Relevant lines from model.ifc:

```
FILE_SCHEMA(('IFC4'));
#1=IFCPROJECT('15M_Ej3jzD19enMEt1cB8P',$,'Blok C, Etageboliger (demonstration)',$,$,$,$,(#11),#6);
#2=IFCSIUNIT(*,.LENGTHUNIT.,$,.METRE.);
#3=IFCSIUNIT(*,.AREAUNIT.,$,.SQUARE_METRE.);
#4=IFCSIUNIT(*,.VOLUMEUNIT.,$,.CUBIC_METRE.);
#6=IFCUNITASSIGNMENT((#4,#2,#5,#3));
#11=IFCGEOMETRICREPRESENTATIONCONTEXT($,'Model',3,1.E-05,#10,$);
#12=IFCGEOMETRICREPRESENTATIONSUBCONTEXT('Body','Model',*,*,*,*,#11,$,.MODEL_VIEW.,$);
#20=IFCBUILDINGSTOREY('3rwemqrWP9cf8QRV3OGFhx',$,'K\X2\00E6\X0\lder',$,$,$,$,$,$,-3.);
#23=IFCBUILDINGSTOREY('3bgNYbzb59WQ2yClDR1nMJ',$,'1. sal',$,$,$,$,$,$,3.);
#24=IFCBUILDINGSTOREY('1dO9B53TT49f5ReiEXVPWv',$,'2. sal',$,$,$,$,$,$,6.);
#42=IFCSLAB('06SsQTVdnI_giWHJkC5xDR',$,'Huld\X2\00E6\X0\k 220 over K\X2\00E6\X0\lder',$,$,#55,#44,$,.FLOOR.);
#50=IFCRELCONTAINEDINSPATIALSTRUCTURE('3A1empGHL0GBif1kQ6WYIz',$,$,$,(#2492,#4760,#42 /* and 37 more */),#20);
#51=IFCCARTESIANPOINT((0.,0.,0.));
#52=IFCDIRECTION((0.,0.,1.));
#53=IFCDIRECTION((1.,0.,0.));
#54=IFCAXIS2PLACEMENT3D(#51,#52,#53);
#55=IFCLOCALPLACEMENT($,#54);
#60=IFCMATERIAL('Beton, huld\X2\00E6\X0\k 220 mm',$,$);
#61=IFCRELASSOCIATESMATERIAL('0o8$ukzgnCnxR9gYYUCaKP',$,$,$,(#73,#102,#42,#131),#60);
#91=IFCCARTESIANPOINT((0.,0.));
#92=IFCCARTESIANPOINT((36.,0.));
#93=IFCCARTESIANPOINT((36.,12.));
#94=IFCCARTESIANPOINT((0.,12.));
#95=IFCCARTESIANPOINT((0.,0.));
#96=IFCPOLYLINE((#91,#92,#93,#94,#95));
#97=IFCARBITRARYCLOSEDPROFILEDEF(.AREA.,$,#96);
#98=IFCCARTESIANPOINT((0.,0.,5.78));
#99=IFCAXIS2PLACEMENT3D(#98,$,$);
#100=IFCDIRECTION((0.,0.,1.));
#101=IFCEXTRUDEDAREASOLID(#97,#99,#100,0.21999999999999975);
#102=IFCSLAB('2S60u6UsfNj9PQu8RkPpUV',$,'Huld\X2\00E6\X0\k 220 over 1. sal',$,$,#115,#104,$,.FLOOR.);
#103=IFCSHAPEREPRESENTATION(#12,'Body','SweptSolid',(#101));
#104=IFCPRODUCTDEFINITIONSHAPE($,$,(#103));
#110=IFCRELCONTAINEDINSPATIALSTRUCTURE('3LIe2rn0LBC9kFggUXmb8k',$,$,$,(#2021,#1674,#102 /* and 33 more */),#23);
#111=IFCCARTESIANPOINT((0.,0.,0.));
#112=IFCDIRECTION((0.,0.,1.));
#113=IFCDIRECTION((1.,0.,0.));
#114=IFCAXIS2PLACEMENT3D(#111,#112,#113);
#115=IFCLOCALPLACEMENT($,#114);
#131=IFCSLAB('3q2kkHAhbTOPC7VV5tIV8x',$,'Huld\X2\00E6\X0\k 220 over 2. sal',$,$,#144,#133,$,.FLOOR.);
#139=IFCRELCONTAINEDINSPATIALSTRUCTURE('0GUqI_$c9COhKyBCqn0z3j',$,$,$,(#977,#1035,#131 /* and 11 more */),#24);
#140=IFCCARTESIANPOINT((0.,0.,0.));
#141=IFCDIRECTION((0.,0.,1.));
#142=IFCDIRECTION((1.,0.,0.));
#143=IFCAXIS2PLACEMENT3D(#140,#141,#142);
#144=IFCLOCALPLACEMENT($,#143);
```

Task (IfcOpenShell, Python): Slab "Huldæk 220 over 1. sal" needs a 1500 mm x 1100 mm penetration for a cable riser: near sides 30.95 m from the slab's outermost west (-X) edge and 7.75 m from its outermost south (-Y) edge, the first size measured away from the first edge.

```python
import numpy as np
import ifcopenshell
import ifcopenshell.api.feature
import ifcopenshell.api.geometry
import ifcopenshell.api.root
import ifcopenshell.geom
import ifcopenshell.util.placement
import ifcopenshell.util.representation
import ifcopenshell.util.shape
import ifcopenshell.util.unit

model = ifcopenshell.open("model.ifc")
unit_scale = ifcopenshell.util.unit.calculate_unit_scale(model)
settings = ifcopenshell.geom.settings()


def volume(element):
    """Net volume in cubic metres, openings subtracted."""
    shape = ifcopenshell.geom.create_shape(settings, element)
    return ifcopenshell.util.shape.get_volume(shape.geometry)


slab = model.by_id(102)
before = volume(slab)

# Extent in the slab's own axes, in metres. The edges named are its -X and -Y sides.
slab_shape = ifcopenshell.geom.create_shape(settings, slab)
vertices = ifcopenshell.util.shape.get_vertices(slab_shape.geometry)
x_min, y_min, bottom = vertices.min(axis=0)
top = vertices[:, 2].max()

opening = ifcopenshell.api.root.create_entity(model, ifc_class="IfcOpeningElement", name="Cable riser opening", predefined_type="OPENING")
context = ifcopenshell.util.representation.get_context(model, "Model", "Body", "MODEL_VIEW")
width, depth = 1.5, 1.1
outline = [(0.0, 0.0), (width, 0.0), (width, depth), (0.0, depth), (0.0, 0.0)]
# Overshoot both faces by 50 mm so the cut is clean.
shape = ifcopenshell.api.geometry.add_slab_representation(
    model, context=context, depth=top - bottom + 0.1, polyline=outline
)
ifcopenshell.api.geometry.assign_representation(model, product=opening, representation=shape)

matrix = ifcopenshell.util.placement.get_local_placement(slab.ObjectPlacement)
matrix[:, 3] = matrix @ np.append(np.array([x_min + 30.95, y_min + 7.75, bottom - 0.05]) / unit_scale, 1.0)
ifcopenshell.api.geometry.edit_object_placement(model, product=opening, matrix=matrix, is_si=False)
ifcopenshell.api.feature.add_feature(model, feature=opening, element=slab)

after = volume(slab)

print(f"slab volume {before:.3f} -> {after:.3f} m3")

model.write("model_edited.ifc")
```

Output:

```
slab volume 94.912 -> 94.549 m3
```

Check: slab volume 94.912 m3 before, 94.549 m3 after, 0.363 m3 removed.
